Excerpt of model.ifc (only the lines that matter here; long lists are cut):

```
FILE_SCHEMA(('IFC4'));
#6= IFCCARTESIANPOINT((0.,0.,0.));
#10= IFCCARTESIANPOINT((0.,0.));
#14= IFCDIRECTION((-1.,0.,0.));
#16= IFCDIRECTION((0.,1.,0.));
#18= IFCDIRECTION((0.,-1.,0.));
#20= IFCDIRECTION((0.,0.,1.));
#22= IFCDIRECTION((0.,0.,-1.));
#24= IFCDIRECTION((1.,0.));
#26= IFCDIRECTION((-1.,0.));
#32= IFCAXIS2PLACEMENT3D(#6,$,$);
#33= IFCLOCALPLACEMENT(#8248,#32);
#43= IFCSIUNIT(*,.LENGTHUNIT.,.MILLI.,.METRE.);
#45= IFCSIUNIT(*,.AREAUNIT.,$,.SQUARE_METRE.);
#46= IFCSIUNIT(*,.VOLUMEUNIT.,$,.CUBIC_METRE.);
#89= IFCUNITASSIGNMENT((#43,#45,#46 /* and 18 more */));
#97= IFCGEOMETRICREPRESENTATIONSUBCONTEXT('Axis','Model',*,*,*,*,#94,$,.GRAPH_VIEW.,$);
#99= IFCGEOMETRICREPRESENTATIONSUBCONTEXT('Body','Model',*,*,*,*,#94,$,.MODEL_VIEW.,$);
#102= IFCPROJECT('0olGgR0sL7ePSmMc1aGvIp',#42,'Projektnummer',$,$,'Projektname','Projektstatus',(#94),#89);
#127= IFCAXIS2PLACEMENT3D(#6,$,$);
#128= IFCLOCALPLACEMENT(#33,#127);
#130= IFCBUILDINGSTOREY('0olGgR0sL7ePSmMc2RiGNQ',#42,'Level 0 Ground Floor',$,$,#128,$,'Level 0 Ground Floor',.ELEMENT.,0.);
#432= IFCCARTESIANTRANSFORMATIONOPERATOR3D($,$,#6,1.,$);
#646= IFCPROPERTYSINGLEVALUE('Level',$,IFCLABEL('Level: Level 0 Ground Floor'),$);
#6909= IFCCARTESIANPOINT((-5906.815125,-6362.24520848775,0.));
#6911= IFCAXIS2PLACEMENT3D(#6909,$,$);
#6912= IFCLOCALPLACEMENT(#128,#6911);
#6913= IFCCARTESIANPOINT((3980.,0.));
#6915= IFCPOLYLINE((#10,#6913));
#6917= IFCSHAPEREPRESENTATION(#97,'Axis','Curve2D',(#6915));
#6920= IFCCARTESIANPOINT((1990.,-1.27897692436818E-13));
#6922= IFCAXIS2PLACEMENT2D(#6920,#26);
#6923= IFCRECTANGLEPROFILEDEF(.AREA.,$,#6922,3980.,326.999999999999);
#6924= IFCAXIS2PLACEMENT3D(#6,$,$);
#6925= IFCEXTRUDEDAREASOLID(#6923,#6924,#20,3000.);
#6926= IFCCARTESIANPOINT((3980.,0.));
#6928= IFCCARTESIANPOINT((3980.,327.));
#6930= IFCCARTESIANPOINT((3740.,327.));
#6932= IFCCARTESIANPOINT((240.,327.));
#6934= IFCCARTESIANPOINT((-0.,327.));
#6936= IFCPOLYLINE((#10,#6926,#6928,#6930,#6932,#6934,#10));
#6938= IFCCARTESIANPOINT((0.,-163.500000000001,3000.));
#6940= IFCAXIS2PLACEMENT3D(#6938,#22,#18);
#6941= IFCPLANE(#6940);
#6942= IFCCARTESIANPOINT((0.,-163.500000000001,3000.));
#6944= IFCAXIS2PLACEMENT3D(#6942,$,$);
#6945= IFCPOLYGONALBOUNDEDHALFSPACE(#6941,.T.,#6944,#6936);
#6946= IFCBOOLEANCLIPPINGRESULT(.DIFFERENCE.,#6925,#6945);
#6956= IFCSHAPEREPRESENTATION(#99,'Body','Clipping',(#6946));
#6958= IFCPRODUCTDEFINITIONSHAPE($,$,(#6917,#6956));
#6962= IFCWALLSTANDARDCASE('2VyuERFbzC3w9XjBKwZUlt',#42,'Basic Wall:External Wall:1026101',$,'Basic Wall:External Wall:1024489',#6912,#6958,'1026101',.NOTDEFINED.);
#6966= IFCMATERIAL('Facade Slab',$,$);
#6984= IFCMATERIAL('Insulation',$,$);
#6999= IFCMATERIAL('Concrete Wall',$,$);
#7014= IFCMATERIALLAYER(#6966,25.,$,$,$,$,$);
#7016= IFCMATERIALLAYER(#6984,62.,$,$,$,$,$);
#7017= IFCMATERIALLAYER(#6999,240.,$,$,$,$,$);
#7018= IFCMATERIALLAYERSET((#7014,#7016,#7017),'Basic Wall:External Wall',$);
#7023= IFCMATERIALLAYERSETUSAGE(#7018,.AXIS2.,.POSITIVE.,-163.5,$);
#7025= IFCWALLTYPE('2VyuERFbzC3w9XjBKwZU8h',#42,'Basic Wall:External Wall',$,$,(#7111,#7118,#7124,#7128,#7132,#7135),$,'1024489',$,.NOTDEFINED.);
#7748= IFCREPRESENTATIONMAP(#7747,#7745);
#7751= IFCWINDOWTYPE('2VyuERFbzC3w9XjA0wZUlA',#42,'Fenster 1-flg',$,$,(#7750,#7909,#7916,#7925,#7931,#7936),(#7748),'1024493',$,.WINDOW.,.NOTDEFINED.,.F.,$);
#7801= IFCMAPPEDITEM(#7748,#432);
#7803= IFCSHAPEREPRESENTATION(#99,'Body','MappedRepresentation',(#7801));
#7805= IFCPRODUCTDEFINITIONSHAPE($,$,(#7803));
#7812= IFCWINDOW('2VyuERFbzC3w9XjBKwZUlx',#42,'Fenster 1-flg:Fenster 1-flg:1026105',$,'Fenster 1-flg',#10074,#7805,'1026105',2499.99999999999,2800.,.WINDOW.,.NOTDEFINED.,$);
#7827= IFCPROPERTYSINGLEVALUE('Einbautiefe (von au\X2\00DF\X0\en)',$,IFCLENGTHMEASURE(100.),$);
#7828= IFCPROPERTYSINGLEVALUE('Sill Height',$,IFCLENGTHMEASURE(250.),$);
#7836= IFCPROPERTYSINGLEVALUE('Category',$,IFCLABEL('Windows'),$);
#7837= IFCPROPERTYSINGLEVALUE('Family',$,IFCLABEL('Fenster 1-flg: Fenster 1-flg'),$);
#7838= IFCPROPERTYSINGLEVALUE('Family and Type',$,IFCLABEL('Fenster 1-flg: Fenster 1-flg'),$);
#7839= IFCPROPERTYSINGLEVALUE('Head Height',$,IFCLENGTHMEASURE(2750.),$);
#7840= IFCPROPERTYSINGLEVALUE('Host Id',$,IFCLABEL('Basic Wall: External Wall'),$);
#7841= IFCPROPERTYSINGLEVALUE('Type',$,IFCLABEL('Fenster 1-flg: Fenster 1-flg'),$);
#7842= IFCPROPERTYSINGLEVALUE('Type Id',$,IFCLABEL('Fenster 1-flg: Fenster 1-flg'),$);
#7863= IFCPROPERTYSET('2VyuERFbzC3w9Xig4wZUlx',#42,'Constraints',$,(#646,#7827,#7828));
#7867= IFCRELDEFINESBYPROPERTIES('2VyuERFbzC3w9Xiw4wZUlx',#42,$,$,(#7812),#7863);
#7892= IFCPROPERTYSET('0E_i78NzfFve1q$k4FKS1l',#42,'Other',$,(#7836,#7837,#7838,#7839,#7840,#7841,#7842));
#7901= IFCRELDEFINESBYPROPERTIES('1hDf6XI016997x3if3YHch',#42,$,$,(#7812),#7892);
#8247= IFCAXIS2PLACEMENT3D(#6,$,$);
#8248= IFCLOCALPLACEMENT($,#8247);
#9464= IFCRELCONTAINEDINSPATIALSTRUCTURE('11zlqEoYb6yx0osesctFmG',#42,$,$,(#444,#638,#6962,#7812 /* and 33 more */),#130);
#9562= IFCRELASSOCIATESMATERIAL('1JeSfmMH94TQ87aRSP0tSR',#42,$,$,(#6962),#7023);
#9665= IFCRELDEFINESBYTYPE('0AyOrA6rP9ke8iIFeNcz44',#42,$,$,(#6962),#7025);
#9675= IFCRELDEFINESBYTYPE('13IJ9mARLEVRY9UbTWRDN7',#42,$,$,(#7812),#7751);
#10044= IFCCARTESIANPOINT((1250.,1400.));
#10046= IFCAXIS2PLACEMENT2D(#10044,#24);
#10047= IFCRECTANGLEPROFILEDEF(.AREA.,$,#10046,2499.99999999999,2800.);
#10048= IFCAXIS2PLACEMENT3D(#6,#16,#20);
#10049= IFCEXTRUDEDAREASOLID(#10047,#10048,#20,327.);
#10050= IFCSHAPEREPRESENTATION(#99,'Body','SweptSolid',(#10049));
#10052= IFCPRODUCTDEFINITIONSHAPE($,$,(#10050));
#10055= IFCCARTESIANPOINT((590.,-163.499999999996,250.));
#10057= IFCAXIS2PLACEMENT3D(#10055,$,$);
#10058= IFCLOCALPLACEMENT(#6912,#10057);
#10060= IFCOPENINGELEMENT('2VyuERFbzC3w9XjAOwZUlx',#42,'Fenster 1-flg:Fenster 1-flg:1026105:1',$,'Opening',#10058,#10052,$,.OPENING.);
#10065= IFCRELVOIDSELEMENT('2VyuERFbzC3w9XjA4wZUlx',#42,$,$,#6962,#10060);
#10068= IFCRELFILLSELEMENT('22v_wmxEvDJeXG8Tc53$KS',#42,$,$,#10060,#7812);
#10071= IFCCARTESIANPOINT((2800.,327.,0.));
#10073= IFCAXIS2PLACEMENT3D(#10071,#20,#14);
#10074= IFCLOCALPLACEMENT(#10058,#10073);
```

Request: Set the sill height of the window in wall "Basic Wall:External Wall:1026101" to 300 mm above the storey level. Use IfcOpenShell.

```python
import numpy as np
import ifcopenshell
import ifcopenshell.api.geometry
import ifcopenshell.api.pset
import ifcopenshell.geom
import ifcopenshell.util.element
import ifcopenshell.util.placement
import ifcopenshell.util.shape
import ifcopenshell.util.unit

model = ifcopenshell.open("model.ifc")
unit_scale = ifcopenshell.util.unit.calculate_unit_scale(model)

window = model.by_guid("2VyuERFbzC3w9XjBKwZUlx")
opening = window.FillsVoids[0].RelatingOpeningElement
storey = ifcopenshell.util.element.get_container(window, ifc_class="IfcBuildingStorey")
level = ifcopenshell.util.placement.get_local_placement(storey.ObjectPlacement)[2, 3]

# The opening's origin need not be at the sill, so measure its lowest point.
shape = ifcopenshell.geom.create_shape(ifcopenshell.geom.settings(), opening)
bottom = ifcopenshell.util.shape.get_shape_bottom_elevation(shape, shape.geometry) / unit_scale
dz = level + 300.0 - bottom

shift = np.array([0.0, 0.0, dz])
# The window is placed relative to its opening, so it follows when the opening moves.
matrix = ifcopenshell.util.placement.get_local_placement(opening.ObjectPlacement)
matrix[:3, 3] += shift
ifcopenshell.api.geometry.edit_object_placement(
    model, product=opening, matrix=matrix, is_si=False, should_transform_children=True
)

# Keep the stored heights in step.
pset = model.by_id(ifcopenshell.util.element.get_pset(window, "Constraints", should_inherit=False)["id"])
ifcopenshell.api.pset.edit_pset(model, pset=pset, properties={
    "Sill Height": model.create_entity("IfcLengthMeasure", ifcopenshell.util.element.get_pset(window, "Constraints", "Sill Height") + dz),
})
pset = model.by_id(ifcopenshell.util.element.get_pset(window, "Other", should_inherit=False)["id"])
ifcopenshell.api.pset.edit_pset(model, pset=pset, properties={
    "Head Height": model.create_entity("IfcLengthMeasure", ifcopenshell.util.element.get_pset(window, "Other", "Head Height") + dz),
})

print(f"moved by {dz * unit_scale:+.3f} m")

model.write("model_rev.ifc")
```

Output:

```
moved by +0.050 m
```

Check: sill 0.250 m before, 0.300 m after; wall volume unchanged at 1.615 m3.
